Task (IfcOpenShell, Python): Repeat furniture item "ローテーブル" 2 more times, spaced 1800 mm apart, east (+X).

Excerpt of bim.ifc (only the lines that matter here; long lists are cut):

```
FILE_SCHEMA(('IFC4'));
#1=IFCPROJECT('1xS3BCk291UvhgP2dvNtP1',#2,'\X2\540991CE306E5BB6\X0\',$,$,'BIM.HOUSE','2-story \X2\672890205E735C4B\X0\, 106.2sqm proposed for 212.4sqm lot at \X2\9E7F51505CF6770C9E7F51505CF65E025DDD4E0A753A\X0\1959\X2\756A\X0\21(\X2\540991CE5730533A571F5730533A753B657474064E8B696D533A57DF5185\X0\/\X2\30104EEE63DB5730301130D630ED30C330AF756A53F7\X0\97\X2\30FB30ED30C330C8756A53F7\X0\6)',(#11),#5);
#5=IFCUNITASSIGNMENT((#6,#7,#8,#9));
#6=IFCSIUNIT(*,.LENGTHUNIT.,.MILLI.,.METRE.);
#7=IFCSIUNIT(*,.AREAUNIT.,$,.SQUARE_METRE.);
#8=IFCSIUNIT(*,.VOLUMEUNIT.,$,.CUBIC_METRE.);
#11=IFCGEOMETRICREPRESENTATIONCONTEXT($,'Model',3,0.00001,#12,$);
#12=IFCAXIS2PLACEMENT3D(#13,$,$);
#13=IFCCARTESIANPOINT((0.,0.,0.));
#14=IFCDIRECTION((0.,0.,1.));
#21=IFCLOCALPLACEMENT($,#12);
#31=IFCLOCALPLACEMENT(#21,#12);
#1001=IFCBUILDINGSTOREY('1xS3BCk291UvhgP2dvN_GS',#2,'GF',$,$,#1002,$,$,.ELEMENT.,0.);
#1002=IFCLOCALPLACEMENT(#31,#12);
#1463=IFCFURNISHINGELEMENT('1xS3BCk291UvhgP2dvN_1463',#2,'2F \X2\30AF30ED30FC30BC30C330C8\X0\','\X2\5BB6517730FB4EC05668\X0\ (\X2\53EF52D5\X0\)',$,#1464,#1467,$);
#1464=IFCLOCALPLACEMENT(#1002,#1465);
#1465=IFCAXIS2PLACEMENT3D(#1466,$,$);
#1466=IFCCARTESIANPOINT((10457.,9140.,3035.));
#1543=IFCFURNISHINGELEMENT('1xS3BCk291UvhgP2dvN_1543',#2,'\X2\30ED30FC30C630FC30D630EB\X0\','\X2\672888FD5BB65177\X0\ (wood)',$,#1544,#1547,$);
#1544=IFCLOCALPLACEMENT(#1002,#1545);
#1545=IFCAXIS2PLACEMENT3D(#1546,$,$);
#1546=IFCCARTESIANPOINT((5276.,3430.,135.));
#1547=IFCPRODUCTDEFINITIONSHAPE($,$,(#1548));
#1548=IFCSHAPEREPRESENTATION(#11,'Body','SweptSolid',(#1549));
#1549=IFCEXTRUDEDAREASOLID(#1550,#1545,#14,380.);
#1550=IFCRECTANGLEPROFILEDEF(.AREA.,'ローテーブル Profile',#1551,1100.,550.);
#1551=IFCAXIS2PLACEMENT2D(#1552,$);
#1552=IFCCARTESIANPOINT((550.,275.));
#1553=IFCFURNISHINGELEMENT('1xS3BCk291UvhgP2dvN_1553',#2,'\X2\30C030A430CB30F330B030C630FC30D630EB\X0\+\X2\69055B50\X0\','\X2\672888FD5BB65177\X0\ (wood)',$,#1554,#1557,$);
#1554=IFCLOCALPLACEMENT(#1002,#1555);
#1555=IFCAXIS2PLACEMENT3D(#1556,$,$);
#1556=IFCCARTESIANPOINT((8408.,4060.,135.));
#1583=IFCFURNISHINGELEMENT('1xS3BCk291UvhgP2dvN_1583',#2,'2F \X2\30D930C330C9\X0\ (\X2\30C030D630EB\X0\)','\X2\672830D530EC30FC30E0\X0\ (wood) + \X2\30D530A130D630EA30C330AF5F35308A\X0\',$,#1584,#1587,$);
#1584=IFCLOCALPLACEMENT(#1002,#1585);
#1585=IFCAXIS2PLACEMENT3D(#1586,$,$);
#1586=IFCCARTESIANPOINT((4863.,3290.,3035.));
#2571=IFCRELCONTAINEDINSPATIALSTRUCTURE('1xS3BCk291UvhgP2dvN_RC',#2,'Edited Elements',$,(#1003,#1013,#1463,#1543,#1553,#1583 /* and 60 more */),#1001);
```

```python
import numpy as np
import ifcopenshell
import ifcopenshell.api.geometry
import ifcopenshell.api.root
import ifcopenshell.util.element
import ifcopenshell.util.placement
import ifcopenshell.util.unit

model = ifcopenshell.open("bim.ifc")
unit_scale = ifcopenshell.util.unit.calculate_unit_scale(model)


def reuse_history(source, copy):
    """copy_class also copies each property set's owner history, people and application; keep the originals."""
    for rel in copy.IsDefinedBy:
        if rel.is_a("IfcRelDefinesByProperties") and (history := rel.RelatingPropertyDefinition.OwnerHistory):
            rel.RelatingPropertyDefinition.OwnerHistory = source.OwnerHistory
            ifcopenshell.util.element.remove_deep2(model, history)


source = model.by_guid("1xS3BCk291UvhgP2dvN_1543")
base = ifcopenshell.util.placement.get_local_placement(source.ObjectPlacement)
step = np.array([1.0, 0.0, 0.0]) * 1.8 / unit_scale

for i in range(1, 3):
    copy = ifcopenshell.api.root.copy_class(model, product=source)
    copy.Representation = ifcopenshell.util.element.copy_deep(
        model, source.Representation, exclude=["IfcGeometricRepresentationContext", "IfcRepresentationMap"]
    )
    reuse_history(source, copy)
    matrix = base.copy()
    matrix[:3, 3] += i * step
    print("added at", matrix[:3, 3].round(3) + 0.0)
    ifcopenshell.api.geometry.edit_object_placement(model, product=copy, matrix=matrix, is_si=False)

model.write("bim-out.ifc")
```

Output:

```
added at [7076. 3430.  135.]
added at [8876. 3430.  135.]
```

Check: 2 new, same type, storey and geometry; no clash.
